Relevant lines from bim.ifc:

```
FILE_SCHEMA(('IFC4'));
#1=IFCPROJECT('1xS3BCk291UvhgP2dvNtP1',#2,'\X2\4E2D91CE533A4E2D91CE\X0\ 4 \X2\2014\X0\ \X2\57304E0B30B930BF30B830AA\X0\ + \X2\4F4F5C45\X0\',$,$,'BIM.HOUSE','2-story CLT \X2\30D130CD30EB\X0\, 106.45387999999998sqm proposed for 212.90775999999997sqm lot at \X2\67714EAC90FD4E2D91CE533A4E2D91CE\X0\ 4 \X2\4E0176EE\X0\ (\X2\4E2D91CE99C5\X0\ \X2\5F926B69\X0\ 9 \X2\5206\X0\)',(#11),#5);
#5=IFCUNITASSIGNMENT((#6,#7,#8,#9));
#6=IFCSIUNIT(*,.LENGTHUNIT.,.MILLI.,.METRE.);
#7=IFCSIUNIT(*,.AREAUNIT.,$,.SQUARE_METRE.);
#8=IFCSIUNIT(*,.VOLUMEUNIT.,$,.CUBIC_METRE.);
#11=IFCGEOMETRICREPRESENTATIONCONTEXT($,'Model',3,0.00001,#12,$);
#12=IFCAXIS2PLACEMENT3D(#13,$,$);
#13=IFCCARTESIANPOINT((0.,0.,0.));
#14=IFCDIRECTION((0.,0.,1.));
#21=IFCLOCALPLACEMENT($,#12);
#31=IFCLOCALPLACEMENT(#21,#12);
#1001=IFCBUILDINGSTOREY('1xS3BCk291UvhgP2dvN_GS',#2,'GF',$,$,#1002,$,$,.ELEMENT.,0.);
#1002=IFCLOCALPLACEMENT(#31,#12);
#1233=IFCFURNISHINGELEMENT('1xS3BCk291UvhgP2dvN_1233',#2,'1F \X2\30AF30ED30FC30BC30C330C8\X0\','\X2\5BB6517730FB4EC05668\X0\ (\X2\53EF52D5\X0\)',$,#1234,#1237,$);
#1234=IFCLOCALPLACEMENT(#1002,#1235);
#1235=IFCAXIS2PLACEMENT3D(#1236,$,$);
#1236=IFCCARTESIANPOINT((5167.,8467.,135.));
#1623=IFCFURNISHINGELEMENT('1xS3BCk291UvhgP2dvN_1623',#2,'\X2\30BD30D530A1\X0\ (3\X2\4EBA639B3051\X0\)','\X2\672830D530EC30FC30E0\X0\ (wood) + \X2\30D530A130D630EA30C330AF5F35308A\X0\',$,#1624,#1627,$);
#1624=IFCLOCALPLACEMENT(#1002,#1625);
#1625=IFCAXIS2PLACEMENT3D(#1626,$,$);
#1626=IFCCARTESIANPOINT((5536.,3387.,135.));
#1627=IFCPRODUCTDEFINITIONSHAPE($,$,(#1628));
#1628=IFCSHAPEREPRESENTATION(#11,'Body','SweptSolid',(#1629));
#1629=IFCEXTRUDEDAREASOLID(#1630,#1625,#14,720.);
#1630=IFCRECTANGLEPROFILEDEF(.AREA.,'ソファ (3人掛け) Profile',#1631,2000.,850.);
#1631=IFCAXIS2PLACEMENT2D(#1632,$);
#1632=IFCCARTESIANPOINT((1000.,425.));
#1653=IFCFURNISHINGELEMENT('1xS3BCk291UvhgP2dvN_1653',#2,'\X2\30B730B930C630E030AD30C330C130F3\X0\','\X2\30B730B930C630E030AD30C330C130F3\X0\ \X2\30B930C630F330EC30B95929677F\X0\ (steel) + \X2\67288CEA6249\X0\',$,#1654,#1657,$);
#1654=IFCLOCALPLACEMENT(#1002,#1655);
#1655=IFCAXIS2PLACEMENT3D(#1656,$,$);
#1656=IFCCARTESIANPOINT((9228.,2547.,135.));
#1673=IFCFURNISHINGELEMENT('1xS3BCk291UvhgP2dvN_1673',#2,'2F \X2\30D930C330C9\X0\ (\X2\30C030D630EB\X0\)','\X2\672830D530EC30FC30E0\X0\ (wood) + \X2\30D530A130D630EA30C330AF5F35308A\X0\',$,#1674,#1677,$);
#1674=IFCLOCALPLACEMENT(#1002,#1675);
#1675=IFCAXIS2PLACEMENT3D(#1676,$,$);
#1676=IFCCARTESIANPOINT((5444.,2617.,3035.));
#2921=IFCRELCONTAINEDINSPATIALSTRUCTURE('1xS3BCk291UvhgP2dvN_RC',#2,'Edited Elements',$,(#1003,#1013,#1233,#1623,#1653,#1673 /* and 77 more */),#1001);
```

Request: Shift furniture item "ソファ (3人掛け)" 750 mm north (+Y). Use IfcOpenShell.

```python
import ifcopenshell
import ifcopenshell.api.geometry
import ifcopenshell.util.placement
import ifcopenshell.util.unit

model = ifcopenshell.open("bim.ifc")
unit_scale = ifcopenshell.util.unit.calculate_unit_scale(model)

item = model.by_guid("1xS3BCk291UvhgP2dvN_1623")
matrix = ifcopenshell.util.placement.get_local_placement(item.ObjectPlacement)
matrix[1, 3] += 0.75 / unit_scale
ifcopenshell.api.geometry.edit_object_placement(model, product=item, matrix=matrix, is_si=False)

print(ifcopenshell.util.placement.get_local_placement(item.ObjectPlacement).round(3) + 0.0)

model.write("bim_updated.ifc")
```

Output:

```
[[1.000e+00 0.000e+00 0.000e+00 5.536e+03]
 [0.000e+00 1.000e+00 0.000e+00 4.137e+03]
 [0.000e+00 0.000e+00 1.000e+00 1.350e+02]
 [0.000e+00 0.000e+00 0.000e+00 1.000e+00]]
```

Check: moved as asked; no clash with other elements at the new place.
